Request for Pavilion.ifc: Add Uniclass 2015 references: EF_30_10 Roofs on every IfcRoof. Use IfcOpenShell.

First a look at what the model holds.

```python
import ifcopenshell

model = ifcopenshell.open("Pavilion.ifc")
print(model.schema)
print("classifications:", [c.Name for c in model.by_type("IfcClassification")])
for ifc_class in ("IfcDoor", "IfcRoof", "IfcStair", "IfcWall", "IfcWindow"):
    print(ifc_class, len(model.by_type(ifc_class)))
```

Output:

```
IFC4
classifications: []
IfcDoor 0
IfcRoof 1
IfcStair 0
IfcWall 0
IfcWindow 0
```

```python
import ifcopenshell
import ifcopenshell.api.classification

model = ifcopenshell.open("Pavilion.ifc")

system = ifcopenshell.api.classification.add_classification(model, classification="Uniclass 2015")

codes = {
    "IfcRoof": ("EF_30_10", "Roofs"),
}
for ifc_class, (code, name) in codes.items():
    products = model.by_type(ifc_class)
    ifcopenshell.api.classification.add_reference(
        model, products=products, classification=system, identification=code, name=name
    )
    print(code, len(products))

model.write("Pavilion-out.ifc")
```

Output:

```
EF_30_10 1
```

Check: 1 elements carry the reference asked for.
